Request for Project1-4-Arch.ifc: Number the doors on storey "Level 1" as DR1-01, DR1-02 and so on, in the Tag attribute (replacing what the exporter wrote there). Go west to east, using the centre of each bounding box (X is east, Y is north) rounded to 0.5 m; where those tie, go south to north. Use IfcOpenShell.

First a look at what the model holds.

```python
import ifcopenshell
import ifcopenshell.util.element
import ifcopenshell.util.placement

model = ifcopenshell.open("Project1-4-Arch.ifc")
print(model.schema)
storey = next(s for s in model.by_type("IfcBuildingStorey") if s.Name == "Level 1")
doors = [e for e in ifcopenshell.util.element.get_decomposition(storey) if e.is_a("IfcDoor")]
for e in sorted(doors, key=lambda e: e.id()):
    origin = ifcopenshell.util.placement.get_local_placement(e.ObjectPlacement)[:3, 3]
    print(e.id(), e.Tag, e.Name, origin.round(2) + 0.0, sep=" | ")
```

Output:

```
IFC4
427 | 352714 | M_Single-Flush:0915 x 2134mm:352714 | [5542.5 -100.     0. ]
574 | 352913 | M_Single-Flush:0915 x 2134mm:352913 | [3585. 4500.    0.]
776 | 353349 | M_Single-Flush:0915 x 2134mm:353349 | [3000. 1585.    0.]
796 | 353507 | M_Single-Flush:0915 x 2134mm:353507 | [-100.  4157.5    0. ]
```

```python
import ifcopenshell
import ifcopenshell.geom
import ifcopenshell.util.element
import ifcopenshell.util.shape

model = ifcopenshell.open("Project1-4-Arch.ifc")
settings = ifcopenshell.geom.settings()
settings.set("use-world-coords", True)


def centre(element):
    shape = ifcopenshell.geom.create_shape(settings, element)
    return ifcopenshell.util.shape.get_bbox_centroid(shape.geometry)


storey = next(s for s in model.by_type("IfcBuildingStorey") if s.Name == "Level 1")
doors = [e for e in ifcopenshell.util.element.get_decomposition(storey) if e.is_a("IfcDoor")]

# Insertion points can sit at a corner or the storey origin, so sort by the geometry (in metres).
centres = {e: centre(e) for e in doors}
doors.sort(key=lambda e: (round(centres[e][0] / 0.5), centres[e][1]))

for i, e in enumerate(doors, start=1):
    number = f"DR1-{i:02d}"
    e.Tag = number
    print(e.id(), number)

model.write("Project1-4-Arch_edited.ifc")
```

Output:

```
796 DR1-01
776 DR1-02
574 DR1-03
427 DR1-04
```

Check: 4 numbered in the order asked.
